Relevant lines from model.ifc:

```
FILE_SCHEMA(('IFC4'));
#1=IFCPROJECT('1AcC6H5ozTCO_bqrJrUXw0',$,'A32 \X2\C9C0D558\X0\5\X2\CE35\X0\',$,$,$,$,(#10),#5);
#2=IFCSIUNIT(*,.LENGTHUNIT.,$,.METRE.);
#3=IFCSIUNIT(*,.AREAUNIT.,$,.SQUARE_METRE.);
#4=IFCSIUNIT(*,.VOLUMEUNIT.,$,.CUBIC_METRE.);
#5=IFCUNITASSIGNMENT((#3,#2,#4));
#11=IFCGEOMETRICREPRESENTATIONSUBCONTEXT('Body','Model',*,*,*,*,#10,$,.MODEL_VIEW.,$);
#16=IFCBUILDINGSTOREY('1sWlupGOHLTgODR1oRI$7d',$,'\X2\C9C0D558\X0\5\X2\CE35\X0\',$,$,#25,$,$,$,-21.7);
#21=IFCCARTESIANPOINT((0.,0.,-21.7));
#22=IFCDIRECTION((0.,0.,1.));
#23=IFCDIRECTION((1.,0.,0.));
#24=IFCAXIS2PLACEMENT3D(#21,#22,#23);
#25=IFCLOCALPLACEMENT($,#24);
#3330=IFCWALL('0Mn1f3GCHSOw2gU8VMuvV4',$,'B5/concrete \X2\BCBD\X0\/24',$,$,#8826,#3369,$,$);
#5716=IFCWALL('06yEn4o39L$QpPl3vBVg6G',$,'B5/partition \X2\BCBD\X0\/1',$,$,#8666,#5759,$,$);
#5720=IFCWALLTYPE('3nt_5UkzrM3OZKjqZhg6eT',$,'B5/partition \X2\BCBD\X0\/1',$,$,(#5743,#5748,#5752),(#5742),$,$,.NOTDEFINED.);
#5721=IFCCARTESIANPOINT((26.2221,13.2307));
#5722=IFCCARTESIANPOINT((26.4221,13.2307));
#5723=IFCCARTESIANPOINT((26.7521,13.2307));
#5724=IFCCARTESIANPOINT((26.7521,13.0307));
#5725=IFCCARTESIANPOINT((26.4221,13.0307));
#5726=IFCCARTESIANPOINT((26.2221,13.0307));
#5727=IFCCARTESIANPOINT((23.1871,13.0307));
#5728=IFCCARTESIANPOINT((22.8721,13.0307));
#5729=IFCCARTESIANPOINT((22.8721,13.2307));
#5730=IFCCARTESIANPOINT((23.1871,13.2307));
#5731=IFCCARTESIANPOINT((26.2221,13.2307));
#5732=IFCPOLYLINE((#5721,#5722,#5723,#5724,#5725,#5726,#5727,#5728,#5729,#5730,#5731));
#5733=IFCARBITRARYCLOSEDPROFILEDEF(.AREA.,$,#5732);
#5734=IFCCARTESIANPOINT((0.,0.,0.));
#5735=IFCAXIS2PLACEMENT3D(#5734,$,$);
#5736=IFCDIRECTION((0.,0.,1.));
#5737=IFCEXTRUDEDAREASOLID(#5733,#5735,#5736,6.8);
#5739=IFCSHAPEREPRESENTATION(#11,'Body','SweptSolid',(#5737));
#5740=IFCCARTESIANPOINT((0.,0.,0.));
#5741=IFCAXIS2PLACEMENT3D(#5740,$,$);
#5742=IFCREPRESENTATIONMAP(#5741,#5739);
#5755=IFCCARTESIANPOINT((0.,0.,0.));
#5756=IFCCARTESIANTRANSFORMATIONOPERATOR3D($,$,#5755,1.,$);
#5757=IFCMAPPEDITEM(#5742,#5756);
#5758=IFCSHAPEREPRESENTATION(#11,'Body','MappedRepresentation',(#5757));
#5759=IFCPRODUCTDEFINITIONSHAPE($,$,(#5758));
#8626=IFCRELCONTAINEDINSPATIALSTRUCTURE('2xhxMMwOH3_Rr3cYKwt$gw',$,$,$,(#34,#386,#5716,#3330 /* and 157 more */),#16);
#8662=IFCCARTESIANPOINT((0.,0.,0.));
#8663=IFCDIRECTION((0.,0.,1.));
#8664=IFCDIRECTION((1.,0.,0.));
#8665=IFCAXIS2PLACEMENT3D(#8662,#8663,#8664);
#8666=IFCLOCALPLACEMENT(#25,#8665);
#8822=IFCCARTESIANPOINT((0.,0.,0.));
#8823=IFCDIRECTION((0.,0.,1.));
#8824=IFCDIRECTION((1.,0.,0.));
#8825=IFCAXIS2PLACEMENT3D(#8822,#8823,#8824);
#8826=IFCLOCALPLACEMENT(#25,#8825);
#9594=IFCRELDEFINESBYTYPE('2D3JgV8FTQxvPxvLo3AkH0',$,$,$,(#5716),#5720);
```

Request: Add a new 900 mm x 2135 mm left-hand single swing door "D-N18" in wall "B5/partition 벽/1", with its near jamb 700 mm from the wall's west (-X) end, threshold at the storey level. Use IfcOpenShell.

```python
import numpy as np
import ifcopenshell
import ifcopenshell.api.feature
import ifcopenshell.api.geometry
import ifcopenshell.api.root
import ifcopenshell.api.spatial
import ifcopenshell.geom
import ifcopenshell.util.element
import ifcopenshell.util.placement
import ifcopenshell.util.representation
import ifcopenshell.util.shape
import ifcopenshell.util.unit

model = ifcopenshell.open("model.ifc")
unit_scale = ifcopenshell.util.unit.calculate_unit_scale(model)
settings = ifcopenshell.geom.settings()


def volume(element):
    """Net volume in cubic metres, openings subtracted."""
    shape = ifcopenshell.geom.create_shape(settings, element)
    return ifcopenshell.util.shape.get_volume(shape.geometry)


wall = model.by_guid("06yEn4o39L$QpPl3vBVg6G")
storey = ifcopenshell.util.element.get_container(wall, ifc_class="IfcBuildingStorey")
context = ifcopenshell.util.representation.get_context(model, "Model", "Body", "MODEL_VIEW")
before = volume(wall)

width, height, from_end, sill = 0.9, 2.135, 0.7, 0.0  # metres

# The wall runs along its own X axis, and the end named is its -X end.
wall_shape = ifcopenshell.geom.create_shape(settings, wall)
x, y, z = ifcopenshell.util.shape.get_vertices(wall_shape.geometry).T
start = x.min() + from_end
face, thickness = float(y.min()), float(y.max() - y.min())
wall_matrix = ifcopenshell.util.placement.get_local_placement(wall.ObjectPlacement)
level = ifcopenshell.util.placement.get_local_placement(storey.ObjectPlacement)[2, 3]


def in_wall(x, y):
    """Placement at x, y metres in the wall's axes, at sill height."""
    matrix = wall_matrix.copy()
    matrix[:, 3] = wall_matrix @ np.array([x / unit_scale, y / unit_scale, 0.0, 1.0])
    matrix[2, 3] = level + sill / unit_scale
    return matrix


# Opening: a box that overshoots both wall faces by 50 mm.
opening = ifcopenshell.api.root.create_entity(model, ifc_class="IfcOpeningElement", predefined_type="OPENING")
box = ifcopenshell.api.geometry.add_wall_representation(
    model, context=context, length=width, height=height, thickness=thickness + 0.1
)
ifcopenshell.api.geometry.assign_representation(model, product=opening, representation=box)
ifcopenshell.api.geometry.edit_object_placement(model, product=opening, matrix=in_wall(start, face - 0.05), is_si=False)
ifcopenshell.api.feature.add_feature(model, feature=opening, element=wall)

door = ifcopenshell.api.root.create_entity(model, ifc_class="IfcDoor", name="D-N18", predefined_type="DOOR")
door.OverallWidth, door.OverallHeight = width / unit_scale, height / unit_scale
door.OperationType = "SINGLE_SWING_LEFT"
body = ifcopenshell.api.geometry.add_door_representation(
    model,
    context=context,
    overall_width=door.OverallWidth,
    overall_height=door.OverallHeight,
    operation_type="SINGLE_SWING_LEFT",
    lining_properties={"LiningDepth": thickness / unit_scale, "ThresholdDepth": thickness / unit_scale},
)
ifcopenshell.api.geometry.assign_representation(model, product=door, representation=body)
ifcopenshell.api.spatial.assign_container(model, products=[door], relating_structure=storey)
ifcopenshell.api.feature.add_filling(model, opening=opening, element=door)

# The lining spans the wall, so the door starts at the wall face.
ifcopenshell.api.geometry.edit_object_placement(model, product=door, matrix=in_wall(start, face), is_si=False)

after = volume(wall)

print(f"wall volume {before:.3f} -> {after:.3f} m3")

model.write("model_rev.ifc")
```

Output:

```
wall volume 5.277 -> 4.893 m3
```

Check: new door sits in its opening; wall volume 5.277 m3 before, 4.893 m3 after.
